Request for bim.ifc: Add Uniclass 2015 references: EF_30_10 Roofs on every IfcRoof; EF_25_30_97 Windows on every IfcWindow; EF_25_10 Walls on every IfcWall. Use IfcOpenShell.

First a look at what the model holds.

```python
import ifcopenshell

model = ifcopenshell.open("bim.ifc")
print(model.schema)
print("classifications:", [c.Name for c in model.by_type("IfcClassification")])
for ifc_class in ("IfcDoor", "IfcRoof", "IfcStair", "IfcWall", "IfcWindow"):
    print(ifc_class, len(model.by_type(ifc_class)))
```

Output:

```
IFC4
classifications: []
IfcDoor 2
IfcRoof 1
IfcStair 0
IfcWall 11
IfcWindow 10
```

```python
import ifcopenshell
import ifcopenshell.api.classification

model = ifcopenshell.open("bim.ifc")

system = ifcopenshell.api.classification.add_classification(model, classification="Uniclass 2015")

codes = {
    "IfcRoof": ("EF_30_10", "Roofs"),
    "IfcWindow": ("EF_25_30_97", "Windows"),
    "IfcWall": ("EF_25_10", "Walls"),
}
for ifc_class, (code, name) in codes.items():
    products = model.by_type(ifc_class)
    ifcopenshell.api.classification.add_reference(
        model, products=products, classification=system, identification=code, name=name
    )
    print(code, len(products))

model.write("bim_updated.ifc")
```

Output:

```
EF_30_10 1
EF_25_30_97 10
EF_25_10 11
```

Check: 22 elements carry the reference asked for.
